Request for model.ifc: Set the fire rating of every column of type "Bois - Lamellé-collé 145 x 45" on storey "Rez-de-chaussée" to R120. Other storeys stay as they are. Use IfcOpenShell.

First a look at what the model holds.

```python
import ifcopenshell
import ifcopenshell.util.element

model = ifcopenshell.open("model.ifc")
print(model.schema)
storey = next(s for s in model.by_type("IfcBuildingStorey") if s.Name == "Rez-de-chaussée")
columns = [e for e in ifcopenshell.util.element.get_decomposition(storey) if e.is_a("IfcColumn")]
seen = {}
for e in columns:
    element_type = ifcopenshell.util.element.get_type(e)
    key = (element_type.Name if element_type != e and element_type else None, ifcopenshell.util.element.get_pset(e, "Pset_ColumnCommon", "FireRating"))
    seen[key] = seen.get(key, 0) + 1
for (name, value), count in sorted(seen.items(), key=str):
    print(count, "x", name, "|", value)
```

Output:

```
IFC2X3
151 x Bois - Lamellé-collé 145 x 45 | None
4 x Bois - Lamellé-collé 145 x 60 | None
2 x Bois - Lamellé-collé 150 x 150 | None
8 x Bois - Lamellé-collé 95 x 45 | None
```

```python
import ifcopenshell
import ifcopenshell.api.pset
import ifcopenshell.util.element

model = ifcopenshell.open("model.ifc")

storey = next(s for s in model.by_type("IfcBuildingStorey") if s.Name == "Rez-de-chaussée")
columns = [e for e in ifcopenshell.util.element.get_decomposition(storey) if e.is_a("IfcColumn")]

count = 0
for e in columns:
    element_type = ifcopenshell.util.element.get_type(e)
    if element_type in (None, e) or element_type.Name != "Bois - Lamellé-collé 145 x 45":
        continue
    # add_pset returns the element's existing set when there is one.
    pset = ifcopenshell.api.pset.add_pset(model, product=e, name="Pset_ColumnCommon")
    ifcopenshell.api.pset.edit_pset(model, pset=pset, properties={"FireRating": "R120"})
    count += 1

print(count, "columns updated")

model.write("model_rev.ifc")
```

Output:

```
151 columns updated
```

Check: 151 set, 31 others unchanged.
